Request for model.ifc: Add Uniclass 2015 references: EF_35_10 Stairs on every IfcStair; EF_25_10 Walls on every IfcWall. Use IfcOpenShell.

First a look at what the model holds.

```python
import ifcopenshell

model = ifcopenshell.open("model.ifc")
print(model.schema)
print("classifications:", [c.Name for c in model.by_type("IfcClassification")])
for ifc_class in ("IfcDoor", "IfcRoof", "IfcStair", "IfcWall", "IfcWindow"):
    print(ifc_class, len(model.by_type(ifc_class)))
```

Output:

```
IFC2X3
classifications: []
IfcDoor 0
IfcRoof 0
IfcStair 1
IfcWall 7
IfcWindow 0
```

```python
import ifcopenshell
import ifcopenshell.api.classification

model = ifcopenshell.open("model.ifc")

# IFC2X3 requires Source and Edition and has no link from the project to the system.
system = model.create_entity("IfcClassification", Source="NBS", Edition="2015", Name="Uniclass 2015")

codes = {
    "IfcStair": ("EF_35_10", "Stairs"),
    "IfcWall": ("EF_25_10", "Walls"),
}
for ifc_class, (code, name) in codes.items():
    products = model.by_type(ifc_class)
    ifcopenshell.api.classification.add_reference(
        model, products=products, classification=system, identification=code, name=name
    )
    print(code, len(products))

model.write("model-out.ifc")
```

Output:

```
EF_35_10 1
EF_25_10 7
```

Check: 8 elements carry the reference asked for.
